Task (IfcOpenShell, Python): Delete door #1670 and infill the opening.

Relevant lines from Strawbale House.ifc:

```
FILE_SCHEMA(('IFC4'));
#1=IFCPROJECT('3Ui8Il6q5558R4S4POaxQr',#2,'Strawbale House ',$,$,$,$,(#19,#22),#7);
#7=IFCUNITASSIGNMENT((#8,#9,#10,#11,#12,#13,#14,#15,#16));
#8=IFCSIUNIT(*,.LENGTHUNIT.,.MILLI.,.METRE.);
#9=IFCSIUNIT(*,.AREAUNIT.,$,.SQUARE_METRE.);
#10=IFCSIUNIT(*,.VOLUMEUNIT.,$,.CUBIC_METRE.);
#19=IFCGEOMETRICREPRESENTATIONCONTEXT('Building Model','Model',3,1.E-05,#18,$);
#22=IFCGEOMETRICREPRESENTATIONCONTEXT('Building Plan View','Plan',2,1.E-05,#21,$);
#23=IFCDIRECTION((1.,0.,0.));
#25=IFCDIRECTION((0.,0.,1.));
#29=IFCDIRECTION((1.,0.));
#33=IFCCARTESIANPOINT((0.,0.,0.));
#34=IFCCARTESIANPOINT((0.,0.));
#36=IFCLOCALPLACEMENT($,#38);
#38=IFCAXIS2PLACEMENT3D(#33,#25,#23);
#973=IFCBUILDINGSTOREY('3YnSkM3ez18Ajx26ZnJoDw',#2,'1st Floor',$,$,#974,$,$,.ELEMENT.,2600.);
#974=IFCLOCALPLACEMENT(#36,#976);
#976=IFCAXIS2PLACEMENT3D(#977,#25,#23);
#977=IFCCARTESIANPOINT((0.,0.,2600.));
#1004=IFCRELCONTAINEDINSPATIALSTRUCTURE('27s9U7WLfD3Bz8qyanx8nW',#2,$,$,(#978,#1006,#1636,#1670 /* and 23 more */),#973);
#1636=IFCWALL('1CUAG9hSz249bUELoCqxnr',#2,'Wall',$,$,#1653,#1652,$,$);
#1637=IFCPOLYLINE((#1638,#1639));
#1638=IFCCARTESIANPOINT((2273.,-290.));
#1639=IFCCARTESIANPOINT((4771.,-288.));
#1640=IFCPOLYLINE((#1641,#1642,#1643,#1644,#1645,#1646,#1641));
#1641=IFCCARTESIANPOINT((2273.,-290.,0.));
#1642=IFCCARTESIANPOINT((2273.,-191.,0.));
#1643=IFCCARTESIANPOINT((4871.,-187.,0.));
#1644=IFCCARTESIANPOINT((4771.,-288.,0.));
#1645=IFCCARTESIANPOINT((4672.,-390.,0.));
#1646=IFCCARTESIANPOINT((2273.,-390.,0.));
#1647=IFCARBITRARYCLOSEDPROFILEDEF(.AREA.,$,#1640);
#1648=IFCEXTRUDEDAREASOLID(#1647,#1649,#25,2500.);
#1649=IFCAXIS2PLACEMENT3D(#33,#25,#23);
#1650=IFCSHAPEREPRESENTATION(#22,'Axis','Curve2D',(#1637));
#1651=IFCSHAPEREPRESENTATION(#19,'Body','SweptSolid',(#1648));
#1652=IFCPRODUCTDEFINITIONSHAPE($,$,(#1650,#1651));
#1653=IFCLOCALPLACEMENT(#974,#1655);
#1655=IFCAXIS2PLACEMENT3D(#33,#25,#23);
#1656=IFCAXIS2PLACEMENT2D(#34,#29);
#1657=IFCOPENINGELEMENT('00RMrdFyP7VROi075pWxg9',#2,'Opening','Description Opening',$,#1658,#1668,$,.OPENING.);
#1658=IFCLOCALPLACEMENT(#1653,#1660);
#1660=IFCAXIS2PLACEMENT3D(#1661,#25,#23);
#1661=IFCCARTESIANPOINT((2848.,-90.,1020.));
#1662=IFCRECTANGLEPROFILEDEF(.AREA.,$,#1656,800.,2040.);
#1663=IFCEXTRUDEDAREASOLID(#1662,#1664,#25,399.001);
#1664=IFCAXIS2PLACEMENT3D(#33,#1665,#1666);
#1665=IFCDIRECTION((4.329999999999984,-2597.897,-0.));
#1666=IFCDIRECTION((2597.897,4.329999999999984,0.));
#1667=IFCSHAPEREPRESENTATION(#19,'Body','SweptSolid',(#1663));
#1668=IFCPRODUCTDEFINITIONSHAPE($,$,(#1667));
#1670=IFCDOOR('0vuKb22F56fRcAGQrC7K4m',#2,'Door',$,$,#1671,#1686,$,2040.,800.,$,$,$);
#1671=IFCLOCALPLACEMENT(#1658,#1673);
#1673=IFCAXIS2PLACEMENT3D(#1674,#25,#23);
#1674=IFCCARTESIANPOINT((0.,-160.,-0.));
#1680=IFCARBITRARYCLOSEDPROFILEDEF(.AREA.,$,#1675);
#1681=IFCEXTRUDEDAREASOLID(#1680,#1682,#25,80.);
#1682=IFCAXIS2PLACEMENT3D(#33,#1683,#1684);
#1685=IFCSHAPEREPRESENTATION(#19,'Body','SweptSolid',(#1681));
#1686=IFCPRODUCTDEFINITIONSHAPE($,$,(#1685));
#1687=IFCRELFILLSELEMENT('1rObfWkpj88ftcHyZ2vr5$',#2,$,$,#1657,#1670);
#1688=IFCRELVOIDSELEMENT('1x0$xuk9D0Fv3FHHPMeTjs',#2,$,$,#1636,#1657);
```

```python
import ifcopenshell
import ifcopenshell.api.feature
import ifcopenshell.api.root
import ifcopenshell.geom
import ifcopenshell.util.shape

model = ifcopenshell.open("Strawbale House.ifc")
settings = ifcopenshell.geom.settings()


def volume(element):
    """Net volume in cubic metres, openings subtracted."""
    shape = ifcopenshell.geom.create_shape(settings, element)
    return ifcopenshell.util.shape.get_volume(shape.geometry)


door = model.by_guid("0vuKb22F56fRcAGQrC7K4m")
opening = door.FillsVoids[0].RelatingOpeningElement
wall = opening.VoidsElements[0].RelatingBuildingElement
before = volume(wall)

ifcopenshell.api.root.remove_product(model, product=door)
ifcopenshell.api.feature.remove_feature(model, feature=opening)

after = volume(wall)

print(f"wall volume {before:.3f} -> {after:.3f} m3")

model.write("Strawbale House_v2.ifc")
```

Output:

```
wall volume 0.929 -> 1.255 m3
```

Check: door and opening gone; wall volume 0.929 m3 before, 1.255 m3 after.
